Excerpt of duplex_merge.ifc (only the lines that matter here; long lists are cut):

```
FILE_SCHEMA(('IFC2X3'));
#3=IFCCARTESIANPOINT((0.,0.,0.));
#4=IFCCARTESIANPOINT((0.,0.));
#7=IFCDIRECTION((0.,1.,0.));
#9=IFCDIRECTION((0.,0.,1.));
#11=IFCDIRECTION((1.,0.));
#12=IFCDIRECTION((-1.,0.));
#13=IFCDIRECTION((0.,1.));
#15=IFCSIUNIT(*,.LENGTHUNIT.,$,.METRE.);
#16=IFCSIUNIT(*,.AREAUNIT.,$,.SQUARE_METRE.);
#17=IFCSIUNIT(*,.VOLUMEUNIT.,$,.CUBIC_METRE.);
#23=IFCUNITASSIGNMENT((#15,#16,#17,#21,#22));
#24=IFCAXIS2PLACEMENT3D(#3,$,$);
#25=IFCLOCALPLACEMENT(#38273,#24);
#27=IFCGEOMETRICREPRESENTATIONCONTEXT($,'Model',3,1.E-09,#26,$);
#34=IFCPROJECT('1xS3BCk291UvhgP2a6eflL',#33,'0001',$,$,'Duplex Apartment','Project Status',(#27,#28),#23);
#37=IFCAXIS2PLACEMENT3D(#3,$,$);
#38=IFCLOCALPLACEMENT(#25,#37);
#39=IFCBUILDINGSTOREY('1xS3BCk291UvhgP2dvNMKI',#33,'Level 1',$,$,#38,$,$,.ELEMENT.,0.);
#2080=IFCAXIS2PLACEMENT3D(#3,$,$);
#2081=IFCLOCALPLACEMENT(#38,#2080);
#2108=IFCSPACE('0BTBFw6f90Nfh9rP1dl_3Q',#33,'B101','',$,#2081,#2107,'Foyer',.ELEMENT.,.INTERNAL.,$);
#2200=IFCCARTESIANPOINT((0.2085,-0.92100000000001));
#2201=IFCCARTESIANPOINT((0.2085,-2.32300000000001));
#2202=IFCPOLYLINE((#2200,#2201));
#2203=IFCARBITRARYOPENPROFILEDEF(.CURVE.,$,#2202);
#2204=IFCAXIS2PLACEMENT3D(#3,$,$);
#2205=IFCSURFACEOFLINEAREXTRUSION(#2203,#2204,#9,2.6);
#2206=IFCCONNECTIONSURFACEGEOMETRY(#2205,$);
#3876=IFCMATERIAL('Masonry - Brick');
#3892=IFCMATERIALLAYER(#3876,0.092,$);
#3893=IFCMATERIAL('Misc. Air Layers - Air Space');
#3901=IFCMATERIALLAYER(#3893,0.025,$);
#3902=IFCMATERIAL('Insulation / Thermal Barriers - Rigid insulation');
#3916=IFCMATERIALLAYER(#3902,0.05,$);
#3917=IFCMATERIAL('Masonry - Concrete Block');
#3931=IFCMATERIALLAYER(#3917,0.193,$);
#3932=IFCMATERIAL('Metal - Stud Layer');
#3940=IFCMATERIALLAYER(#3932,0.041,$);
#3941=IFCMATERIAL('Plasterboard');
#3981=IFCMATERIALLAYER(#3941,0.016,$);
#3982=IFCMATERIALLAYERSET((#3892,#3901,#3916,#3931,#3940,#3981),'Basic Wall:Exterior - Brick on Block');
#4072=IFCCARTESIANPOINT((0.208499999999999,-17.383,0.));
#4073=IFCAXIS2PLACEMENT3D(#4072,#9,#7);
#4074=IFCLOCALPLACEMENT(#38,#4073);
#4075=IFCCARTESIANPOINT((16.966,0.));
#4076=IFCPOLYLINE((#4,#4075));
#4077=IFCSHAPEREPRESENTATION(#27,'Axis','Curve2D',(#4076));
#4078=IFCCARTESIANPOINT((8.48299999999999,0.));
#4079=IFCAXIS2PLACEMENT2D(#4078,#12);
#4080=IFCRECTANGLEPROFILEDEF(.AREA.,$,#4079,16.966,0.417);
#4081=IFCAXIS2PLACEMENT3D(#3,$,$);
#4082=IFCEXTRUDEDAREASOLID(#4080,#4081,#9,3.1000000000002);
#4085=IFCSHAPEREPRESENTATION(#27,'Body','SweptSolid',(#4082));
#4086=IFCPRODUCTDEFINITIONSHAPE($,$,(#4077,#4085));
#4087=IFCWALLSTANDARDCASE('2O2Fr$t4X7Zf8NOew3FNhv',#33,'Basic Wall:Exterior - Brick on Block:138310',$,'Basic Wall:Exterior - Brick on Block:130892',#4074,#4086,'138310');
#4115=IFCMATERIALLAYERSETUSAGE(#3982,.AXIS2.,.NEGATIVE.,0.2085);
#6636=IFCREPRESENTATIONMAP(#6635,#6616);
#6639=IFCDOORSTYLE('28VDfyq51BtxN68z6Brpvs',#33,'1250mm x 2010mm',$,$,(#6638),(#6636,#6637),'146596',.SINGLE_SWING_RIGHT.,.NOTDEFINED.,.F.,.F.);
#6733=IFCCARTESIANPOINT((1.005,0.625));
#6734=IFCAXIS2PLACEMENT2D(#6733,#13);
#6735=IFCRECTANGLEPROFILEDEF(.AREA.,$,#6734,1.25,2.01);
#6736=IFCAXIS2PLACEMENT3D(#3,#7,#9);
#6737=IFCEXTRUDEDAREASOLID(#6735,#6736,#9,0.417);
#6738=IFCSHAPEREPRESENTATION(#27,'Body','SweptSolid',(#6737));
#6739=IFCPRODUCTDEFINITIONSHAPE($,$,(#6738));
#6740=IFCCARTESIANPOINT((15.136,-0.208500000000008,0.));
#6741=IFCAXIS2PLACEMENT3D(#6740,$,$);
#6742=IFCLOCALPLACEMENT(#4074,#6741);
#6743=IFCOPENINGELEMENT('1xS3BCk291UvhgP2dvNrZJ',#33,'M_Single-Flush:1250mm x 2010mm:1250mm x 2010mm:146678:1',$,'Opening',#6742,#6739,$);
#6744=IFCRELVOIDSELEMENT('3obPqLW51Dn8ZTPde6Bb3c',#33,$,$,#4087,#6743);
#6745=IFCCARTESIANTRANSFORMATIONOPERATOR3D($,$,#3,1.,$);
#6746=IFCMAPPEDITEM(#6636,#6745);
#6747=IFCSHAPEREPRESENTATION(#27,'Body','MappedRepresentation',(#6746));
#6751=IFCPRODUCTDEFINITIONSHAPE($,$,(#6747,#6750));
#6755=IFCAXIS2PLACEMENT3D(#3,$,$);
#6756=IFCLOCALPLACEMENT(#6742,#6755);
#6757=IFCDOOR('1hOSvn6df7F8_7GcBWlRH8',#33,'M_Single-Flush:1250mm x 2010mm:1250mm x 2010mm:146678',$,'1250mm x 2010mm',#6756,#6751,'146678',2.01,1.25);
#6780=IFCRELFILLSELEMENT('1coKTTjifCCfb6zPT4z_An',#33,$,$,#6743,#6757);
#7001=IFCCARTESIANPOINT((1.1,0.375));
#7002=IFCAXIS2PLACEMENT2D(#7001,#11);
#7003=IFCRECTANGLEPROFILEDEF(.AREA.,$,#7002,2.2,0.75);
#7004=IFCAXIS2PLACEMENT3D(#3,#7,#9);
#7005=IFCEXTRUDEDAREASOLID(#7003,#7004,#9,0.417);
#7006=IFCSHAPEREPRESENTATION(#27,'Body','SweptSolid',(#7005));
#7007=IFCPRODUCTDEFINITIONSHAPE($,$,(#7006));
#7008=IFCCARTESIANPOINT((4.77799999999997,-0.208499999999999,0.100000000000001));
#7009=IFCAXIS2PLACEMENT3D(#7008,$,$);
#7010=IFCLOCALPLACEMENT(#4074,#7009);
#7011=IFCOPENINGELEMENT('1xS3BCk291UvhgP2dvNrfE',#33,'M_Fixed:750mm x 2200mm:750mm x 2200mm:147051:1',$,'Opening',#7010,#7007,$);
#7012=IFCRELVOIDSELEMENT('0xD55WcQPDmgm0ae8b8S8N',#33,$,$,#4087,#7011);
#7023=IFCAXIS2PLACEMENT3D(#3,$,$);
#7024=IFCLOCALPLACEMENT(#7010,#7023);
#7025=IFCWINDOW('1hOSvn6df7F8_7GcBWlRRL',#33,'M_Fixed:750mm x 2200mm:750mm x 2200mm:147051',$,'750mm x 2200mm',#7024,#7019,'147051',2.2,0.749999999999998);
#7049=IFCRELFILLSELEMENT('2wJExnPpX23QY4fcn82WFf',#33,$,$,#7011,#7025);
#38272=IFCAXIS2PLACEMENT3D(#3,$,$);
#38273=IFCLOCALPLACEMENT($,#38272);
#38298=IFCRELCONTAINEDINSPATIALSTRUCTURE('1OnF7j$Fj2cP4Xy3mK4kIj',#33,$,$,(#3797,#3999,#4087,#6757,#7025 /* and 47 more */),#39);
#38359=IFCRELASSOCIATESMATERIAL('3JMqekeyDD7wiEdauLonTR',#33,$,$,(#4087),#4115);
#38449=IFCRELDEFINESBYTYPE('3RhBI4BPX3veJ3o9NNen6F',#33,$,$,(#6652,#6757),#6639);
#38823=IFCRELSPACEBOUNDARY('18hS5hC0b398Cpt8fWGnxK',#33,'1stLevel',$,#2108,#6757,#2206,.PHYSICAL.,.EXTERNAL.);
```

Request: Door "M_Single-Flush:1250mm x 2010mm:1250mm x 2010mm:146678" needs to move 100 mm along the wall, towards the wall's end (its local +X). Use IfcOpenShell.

```python
import numpy as np
import ifcopenshell
import ifcopenshell.api.geometry
import ifcopenshell.util.placement

model = ifcopenshell.open("duplex_merge.ifc")

door = model.by_guid("1hOSvn6df7F8_7GcBWlRH8")
opening = door.FillsVoids[0].RelatingOpeningElement
wall = opening.VoidsElements[0].RelatingBuildingElement

wall_matrix = ifcopenshell.util.placement.get_local_placement(wall.ObjectPlacement)
shift = wall_matrix[:3, 0] * 0.1
before = ifcopenshell.util.placement.get_local_placement(door.ObjectPlacement)[:3, 3].copy()

# The door is placed relative to its opening, so it follows when the opening moves.
matrix = ifcopenshell.util.placement.get_local_placement(opening.ObjectPlacement)
matrix[:3, 3] += shift
ifcopenshell.api.geometry.edit_object_placement(
    model, product=opening, matrix=matrix, is_si=False, should_transform_children=True
)

# Space boundary surfaces are stored in each space's coordinates; move them too.
for rel in door.ProvidesBoundaries:
    if not rel.ConnectionGeometry:
        continue
    surface = rel.ConnectionGeometry.SurfaceOnRelatingElement
    space_matrix = ifcopenshell.util.placement.get_local_placement(rel.RelatingSpace.ObjectPlacement)
    point = np.array(surface.Position.Location.Coordinates) + space_matrix[:3, :3].T @ shift
    surface.Position = model.createIfcAxis2Placement3D(
        model.createIfcCartesianPoint(point.tolist()), surface.Position.Axis, surface.Position.RefDirection
    )

after = ifcopenshell.util.placement.get_local_placement(door.ObjectPlacement)[:3, 3]
print("door moved by", (after - before).round(3) + 0.0)

model.write("duplex_merge_updated.ifc")
```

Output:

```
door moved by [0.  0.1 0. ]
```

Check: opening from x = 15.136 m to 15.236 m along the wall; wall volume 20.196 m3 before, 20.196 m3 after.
